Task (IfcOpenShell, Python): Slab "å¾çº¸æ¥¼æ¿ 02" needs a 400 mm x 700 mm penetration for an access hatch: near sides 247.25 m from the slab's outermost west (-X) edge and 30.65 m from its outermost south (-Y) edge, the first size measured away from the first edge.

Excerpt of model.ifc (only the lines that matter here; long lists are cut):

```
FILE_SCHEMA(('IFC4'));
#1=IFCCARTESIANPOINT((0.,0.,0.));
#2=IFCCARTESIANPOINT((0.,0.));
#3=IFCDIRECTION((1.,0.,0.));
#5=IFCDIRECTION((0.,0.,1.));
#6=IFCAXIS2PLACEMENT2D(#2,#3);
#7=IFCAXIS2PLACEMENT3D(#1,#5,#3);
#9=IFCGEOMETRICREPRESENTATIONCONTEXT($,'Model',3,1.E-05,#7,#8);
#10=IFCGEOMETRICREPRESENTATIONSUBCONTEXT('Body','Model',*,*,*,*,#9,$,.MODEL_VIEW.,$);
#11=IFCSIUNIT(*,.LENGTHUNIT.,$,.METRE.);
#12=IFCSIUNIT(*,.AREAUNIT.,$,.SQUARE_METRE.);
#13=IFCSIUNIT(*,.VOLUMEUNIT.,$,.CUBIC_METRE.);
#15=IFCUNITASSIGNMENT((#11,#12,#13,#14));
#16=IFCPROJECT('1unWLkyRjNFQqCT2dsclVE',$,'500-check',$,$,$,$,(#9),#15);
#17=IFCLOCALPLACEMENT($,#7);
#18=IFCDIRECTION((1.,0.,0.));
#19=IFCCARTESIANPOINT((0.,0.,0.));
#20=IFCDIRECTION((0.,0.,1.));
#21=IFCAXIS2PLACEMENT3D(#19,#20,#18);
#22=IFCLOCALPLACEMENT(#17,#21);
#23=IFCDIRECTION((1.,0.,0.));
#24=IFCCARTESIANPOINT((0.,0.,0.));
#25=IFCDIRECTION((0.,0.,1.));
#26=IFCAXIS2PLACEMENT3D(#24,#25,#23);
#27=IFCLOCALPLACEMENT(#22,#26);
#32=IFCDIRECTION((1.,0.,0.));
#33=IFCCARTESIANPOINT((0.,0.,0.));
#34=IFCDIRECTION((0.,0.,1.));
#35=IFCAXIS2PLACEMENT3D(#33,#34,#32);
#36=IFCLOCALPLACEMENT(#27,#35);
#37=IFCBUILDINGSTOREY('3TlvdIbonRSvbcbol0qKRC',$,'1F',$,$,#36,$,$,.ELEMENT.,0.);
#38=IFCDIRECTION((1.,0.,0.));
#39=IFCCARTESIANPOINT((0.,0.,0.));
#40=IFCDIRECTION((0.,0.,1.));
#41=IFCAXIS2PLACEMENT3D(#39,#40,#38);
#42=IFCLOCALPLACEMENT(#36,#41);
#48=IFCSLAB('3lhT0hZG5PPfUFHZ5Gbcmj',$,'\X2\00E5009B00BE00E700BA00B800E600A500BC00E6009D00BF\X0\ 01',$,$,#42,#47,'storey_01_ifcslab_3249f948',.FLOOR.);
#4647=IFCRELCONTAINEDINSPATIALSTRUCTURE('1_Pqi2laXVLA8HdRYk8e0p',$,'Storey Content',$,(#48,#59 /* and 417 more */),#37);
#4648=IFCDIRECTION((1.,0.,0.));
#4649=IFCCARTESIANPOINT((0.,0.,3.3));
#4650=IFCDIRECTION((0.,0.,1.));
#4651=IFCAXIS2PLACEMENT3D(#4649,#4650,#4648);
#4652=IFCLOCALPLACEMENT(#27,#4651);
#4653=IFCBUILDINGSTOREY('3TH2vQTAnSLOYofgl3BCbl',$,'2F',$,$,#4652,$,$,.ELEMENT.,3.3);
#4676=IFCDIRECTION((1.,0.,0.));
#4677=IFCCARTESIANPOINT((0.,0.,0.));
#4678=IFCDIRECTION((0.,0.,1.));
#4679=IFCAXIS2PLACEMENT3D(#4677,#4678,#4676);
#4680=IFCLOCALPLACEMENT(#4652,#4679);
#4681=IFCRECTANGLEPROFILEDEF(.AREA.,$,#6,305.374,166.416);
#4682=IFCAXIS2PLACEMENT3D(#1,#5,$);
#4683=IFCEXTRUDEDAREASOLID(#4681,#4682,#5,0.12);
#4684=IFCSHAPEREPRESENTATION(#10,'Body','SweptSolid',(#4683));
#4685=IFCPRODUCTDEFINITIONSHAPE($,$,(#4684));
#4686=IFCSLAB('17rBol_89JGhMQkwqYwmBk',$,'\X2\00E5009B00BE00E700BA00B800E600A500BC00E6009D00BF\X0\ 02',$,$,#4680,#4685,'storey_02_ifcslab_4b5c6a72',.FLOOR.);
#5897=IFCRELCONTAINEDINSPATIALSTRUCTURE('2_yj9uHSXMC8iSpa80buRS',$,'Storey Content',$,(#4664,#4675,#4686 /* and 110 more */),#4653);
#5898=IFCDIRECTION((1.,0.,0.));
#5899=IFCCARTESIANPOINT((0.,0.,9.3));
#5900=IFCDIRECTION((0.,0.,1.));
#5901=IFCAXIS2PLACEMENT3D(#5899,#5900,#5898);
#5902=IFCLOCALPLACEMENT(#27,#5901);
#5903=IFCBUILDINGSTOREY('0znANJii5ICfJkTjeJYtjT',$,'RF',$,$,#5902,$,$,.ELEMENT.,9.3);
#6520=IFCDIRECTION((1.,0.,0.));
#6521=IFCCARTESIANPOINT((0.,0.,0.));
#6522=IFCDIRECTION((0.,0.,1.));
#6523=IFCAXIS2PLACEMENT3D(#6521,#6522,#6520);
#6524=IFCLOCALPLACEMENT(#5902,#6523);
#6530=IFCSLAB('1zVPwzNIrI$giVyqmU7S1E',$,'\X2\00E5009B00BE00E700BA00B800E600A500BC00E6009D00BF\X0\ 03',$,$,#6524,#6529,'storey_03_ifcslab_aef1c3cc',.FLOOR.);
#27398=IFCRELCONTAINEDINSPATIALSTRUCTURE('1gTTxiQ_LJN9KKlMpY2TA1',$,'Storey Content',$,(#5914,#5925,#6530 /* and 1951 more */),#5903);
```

```python
import numpy as np
import ifcopenshell
import ifcopenshell.api.feature
import ifcopenshell.api.geometry
import ifcopenshell.api.root
import ifcopenshell.geom
import ifcopenshell.util.placement
import ifcopenshell.util.representation
import ifcopenshell.util.shape
import ifcopenshell.util.unit

model = ifcopenshell.open("model.ifc")
unit_scale = ifcopenshell.util.unit.calculate_unit_scale(model)
settings = ifcopenshell.geom.settings()


def volume(element):
    """Net volume in cubic metres, openings subtracted."""
    shape = ifcopenshell.geom.create_shape(settings, element)
    return ifcopenshell.util.shape.get_volume(shape.geometry)


slab = model.by_guid("17rBol_89JGhMQkwqYwmBk")
before = volume(slab)

# Extent in the slab's own axes, in metres. The edges named are its -X and -Y sides.
slab_shape = ifcopenshell.geom.create_shape(settings, slab)
vertices = ifcopenshell.util.shape.get_vertices(slab_shape.geometry)
x_min, y_min, bottom = vertices.min(axis=0)
top = vertices[:, 2].max()

opening = ifcopenshell.api.root.create_entity(model, ifc_class="IfcOpeningElement", name="Access hatch opening", predefined_type="OPENING")
context = ifcopenshell.util.representation.get_context(model, "Model", "Body", "MODEL_VIEW")
width, depth = 0.4, 0.7
outline = [(0.0, 0.0), (width, 0.0), (width, depth), (0.0, depth), (0.0, 0.0)]
# Overshoot both faces by 50 mm so the cut is clean.
shape = ifcopenshell.api.geometry.add_slab_representation(
    model, context=context, depth=top - bottom + 0.1, polyline=outline
)
ifcopenshell.api.geometry.assign_representation(model, product=opening, representation=shape)

matrix = ifcopenshell.util.placement.get_local_placement(slab.ObjectPlacement)
matrix[:, 3] = matrix @ np.append(np.array([x_min + 247.25, y_min + 30.65, bottom - 0.05]) / unit_scale, 1.0)
ifcopenshell.api.geometry.edit_object_placement(model, product=opening, matrix=matrix, is_si=False)
ifcopenshell.api.feature.add_feature(model, feature=opening, element=slab)

after = volume(slab)

print(f"slab volume {before:.3f} -> {after:.3f} m3")

model.write("model_updated.ifc")
```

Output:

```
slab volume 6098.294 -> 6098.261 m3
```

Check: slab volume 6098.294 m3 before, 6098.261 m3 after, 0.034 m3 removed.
